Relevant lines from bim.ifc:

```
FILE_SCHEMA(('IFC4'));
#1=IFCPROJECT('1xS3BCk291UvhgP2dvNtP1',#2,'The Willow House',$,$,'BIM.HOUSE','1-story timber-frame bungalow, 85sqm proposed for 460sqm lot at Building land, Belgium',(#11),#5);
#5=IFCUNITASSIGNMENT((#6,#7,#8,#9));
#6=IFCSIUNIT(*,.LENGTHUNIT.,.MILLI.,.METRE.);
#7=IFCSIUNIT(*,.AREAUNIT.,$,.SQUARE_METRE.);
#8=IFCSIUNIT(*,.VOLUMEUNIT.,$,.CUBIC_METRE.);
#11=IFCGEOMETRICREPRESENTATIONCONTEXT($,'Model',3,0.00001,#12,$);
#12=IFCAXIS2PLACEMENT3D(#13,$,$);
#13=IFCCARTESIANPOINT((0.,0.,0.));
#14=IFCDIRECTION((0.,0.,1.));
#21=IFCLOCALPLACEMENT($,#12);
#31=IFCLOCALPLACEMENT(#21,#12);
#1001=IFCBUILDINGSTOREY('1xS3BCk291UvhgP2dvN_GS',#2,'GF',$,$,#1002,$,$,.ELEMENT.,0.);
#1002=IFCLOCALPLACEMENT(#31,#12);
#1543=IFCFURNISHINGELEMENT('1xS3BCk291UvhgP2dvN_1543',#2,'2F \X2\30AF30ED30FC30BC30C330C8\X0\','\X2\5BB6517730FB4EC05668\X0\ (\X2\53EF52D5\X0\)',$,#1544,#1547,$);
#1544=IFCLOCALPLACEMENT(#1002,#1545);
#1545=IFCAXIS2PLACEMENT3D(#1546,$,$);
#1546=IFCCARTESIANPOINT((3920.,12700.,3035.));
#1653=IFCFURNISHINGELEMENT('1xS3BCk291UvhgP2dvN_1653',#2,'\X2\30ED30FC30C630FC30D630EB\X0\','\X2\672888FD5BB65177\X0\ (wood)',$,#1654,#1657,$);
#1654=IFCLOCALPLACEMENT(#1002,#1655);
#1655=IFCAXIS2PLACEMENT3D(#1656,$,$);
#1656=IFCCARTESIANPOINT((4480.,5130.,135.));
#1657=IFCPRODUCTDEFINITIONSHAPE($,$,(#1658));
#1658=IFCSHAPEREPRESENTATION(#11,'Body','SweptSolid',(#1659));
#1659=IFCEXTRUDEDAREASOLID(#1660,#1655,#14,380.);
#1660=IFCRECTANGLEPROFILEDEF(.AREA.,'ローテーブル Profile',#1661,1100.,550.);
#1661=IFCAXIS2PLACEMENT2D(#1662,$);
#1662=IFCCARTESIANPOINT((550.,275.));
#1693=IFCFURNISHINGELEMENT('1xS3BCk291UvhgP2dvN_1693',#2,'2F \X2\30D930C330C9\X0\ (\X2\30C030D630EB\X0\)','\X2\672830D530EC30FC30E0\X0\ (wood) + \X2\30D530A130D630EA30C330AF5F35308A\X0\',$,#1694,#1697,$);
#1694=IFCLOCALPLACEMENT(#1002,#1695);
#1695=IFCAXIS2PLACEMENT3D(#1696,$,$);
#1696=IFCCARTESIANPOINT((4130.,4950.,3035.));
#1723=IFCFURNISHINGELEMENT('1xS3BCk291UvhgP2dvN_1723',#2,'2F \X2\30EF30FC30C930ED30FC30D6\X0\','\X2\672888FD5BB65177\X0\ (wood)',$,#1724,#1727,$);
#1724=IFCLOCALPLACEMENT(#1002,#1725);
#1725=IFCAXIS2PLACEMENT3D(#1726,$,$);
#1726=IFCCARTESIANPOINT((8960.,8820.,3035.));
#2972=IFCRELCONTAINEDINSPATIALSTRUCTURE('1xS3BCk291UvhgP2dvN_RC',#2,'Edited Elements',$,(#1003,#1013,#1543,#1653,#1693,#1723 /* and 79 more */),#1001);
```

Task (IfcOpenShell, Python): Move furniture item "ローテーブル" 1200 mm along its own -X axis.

```python
import ifcopenshell
import ifcopenshell.api.geometry
import ifcopenshell.util.placement
import ifcopenshell.util.unit

model = ifcopenshell.open("bim.ifc")
unit_scale = ifcopenshell.util.unit.calculate_unit_scale(model)

item = model.by_guid("1xS3BCk291UvhgP2dvN_1653")
matrix = ifcopenshell.util.placement.get_local_placement(item.ObjectPlacement)
matrix[:3, 3] -= matrix[:3, 0] * 1.2 / unit_scale
ifcopenshell.api.geometry.edit_object_placement(model, product=item, matrix=matrix, is_si=False)

print(ifcopenshell.util.placement.get_local_placement(item.ObjectPlacement).round(3) + 0.0)

model.write("bim_updated.ifc")
```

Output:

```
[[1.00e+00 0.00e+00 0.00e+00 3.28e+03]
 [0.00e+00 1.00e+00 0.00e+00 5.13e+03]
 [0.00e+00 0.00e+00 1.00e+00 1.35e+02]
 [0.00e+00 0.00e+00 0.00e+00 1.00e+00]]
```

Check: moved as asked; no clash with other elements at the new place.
